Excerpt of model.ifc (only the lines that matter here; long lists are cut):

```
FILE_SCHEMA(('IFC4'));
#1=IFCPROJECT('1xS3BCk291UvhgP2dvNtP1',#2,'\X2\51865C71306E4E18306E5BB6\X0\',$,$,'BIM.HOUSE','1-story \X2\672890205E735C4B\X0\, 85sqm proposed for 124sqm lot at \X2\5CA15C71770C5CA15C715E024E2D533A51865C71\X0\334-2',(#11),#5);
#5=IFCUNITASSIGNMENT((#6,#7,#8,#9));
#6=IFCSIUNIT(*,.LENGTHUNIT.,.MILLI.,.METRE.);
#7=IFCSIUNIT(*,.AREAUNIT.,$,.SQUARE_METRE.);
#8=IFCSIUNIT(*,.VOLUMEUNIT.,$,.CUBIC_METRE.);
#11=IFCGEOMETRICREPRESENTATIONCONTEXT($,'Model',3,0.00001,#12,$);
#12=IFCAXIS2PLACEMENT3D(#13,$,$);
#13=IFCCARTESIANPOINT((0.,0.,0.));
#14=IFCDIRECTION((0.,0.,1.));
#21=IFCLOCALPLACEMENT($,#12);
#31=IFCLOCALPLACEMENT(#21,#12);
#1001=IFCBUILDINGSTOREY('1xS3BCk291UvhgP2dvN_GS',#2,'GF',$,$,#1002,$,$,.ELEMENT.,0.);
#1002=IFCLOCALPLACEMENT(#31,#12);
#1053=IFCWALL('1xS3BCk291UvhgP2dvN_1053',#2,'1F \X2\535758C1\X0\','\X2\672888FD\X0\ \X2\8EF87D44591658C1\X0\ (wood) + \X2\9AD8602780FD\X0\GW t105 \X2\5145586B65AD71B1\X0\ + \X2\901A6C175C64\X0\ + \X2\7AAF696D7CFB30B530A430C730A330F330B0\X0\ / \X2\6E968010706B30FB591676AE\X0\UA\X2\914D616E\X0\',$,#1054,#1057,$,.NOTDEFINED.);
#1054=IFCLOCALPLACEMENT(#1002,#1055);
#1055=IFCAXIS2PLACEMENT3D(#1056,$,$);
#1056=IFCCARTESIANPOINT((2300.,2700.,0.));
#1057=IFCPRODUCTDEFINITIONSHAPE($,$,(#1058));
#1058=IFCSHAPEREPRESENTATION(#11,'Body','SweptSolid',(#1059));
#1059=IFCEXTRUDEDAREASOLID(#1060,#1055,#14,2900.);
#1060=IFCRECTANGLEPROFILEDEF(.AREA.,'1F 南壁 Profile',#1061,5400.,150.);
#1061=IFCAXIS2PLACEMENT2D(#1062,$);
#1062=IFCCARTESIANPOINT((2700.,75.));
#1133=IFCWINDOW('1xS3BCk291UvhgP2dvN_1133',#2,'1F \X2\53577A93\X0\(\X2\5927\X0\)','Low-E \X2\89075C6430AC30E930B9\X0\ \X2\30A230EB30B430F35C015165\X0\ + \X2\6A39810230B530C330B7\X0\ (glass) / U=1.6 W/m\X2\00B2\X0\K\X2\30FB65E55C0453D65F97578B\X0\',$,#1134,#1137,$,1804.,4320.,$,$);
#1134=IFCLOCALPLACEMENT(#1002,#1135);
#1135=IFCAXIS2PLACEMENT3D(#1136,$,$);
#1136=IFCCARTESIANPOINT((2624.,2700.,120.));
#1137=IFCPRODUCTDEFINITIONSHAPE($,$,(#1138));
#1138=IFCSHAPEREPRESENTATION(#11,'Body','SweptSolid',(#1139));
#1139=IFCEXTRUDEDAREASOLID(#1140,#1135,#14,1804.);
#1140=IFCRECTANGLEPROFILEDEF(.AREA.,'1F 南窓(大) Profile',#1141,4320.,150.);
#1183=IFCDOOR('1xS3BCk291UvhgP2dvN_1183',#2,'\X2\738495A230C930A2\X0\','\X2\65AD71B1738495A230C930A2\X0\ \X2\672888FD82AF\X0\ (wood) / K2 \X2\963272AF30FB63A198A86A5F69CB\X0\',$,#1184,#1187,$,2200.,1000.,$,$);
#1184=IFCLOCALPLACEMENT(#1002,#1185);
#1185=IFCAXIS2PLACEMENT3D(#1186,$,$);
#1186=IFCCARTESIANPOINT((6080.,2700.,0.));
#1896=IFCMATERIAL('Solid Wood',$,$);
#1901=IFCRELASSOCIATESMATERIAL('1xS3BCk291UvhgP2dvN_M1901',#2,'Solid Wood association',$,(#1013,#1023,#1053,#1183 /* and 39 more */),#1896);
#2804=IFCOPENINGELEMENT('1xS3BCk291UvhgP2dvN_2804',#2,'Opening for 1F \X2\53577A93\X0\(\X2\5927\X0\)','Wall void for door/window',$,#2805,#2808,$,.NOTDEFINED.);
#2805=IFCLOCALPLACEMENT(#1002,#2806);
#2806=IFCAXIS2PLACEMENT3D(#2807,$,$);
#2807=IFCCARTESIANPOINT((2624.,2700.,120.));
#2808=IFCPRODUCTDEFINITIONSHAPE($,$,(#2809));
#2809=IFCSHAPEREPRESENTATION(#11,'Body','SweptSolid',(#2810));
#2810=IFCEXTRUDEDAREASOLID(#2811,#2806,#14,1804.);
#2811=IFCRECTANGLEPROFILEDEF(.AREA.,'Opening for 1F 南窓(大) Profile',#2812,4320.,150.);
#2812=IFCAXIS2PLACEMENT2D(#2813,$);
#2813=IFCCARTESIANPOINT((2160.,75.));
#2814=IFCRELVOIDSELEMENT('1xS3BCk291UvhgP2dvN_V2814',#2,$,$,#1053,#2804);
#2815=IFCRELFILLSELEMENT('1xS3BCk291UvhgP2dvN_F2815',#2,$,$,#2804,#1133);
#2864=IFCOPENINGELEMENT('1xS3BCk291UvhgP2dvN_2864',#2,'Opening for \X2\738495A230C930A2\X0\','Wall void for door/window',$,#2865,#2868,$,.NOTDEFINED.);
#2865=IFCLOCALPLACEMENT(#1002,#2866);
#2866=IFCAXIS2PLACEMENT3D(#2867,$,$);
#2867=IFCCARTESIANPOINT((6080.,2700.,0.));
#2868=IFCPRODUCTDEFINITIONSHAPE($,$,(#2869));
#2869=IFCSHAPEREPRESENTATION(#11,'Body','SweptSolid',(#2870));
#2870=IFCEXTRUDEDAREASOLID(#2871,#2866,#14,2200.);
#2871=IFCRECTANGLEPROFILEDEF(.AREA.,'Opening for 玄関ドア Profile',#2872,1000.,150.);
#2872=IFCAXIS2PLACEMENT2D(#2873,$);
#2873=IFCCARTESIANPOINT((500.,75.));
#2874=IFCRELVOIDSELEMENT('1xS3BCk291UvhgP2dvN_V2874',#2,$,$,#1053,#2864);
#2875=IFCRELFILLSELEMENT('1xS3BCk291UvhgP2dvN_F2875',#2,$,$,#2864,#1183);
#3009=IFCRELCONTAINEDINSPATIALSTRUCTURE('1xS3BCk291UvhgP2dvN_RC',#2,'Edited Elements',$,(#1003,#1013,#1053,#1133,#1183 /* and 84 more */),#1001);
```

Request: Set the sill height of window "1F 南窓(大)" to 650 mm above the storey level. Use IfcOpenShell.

```python
import numpy as np
import ifcopenshell
import ifcopenshell.api.geometry
import ifcopenshell.geom
import ifcopenshell.util.element
import ifcopenshell.util.placement
import ifcopenshell.util.shape
import ifcopenshell.util.unit

model = ifcopenshell.open("model.ifc")
unit_scale = ifcopenshell.util.unit.calculate_unit_scale(model)

window = model.by_id(1133)
opening = window.FillsVoids[0].RelatingOpeningElement
storey = ifcopenshell.util.element.get_container(window, ifc_class="IfcBuildingStorey")
level = ifcopenshell.util.placement.get_local_placement(storey.ObjectPlacement)[2, 3]

# The opening's origin need not be at the sill, so measure its lowest point.
shape = ifcopenshell.geom.create_shape(ifcopenshell.geom.settings(), opening)
bottom = ifcopenshell.util.shape.get_shape_bottom_elevation(shape, shape.geometry) / unit_scale
dz = level + 0.65 / unit_scale - bottom

shift = np.array([0.0, 0.0, dz])
# The window is not placed relative to its opening, so move both.
for product in (opening, window):
    matrix = ifcopenshell.util.placement.get_local_placement(product.ObjectPlacement)
    matrix[:3, 3] += shift
    ifcopenshell.api.geometry.edit_object_placement(model, product=product, matrix=matrix, is_si=False)

print(f"moved by {dz * unit_scale:+.3f} m")

model.write("model-out.ifc")
```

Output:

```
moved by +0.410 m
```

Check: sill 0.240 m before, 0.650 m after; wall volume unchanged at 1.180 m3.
